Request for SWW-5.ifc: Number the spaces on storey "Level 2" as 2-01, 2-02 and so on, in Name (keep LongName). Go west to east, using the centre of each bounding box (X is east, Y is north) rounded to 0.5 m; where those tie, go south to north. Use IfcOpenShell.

First a look at what the model holds.

```python
import ifcopenshell
import ifcopenshell.util.element
import ifcopenshell.util.placement

model = ifcopenshell.open("SWW-5.ifc")
print(model.schema)
storey = next(s for s in model.by_type("IfcBuildingStorey") if s.Name == "Level 2")
spaces = [e for e in ifcopenshell.util.element.get_decomposition(storey) if e.is_a("IfcSpace")]
for e in sorted(spaces, key=lambda e: e.id()):
    origin = ifcopenshell.util.placement.get_local_placement(e.ObjectPlacement)[:3, 3]
    print(e.id(), e.Name, e.LongName, origin.round(2) + 0.0, sep=" | ")
```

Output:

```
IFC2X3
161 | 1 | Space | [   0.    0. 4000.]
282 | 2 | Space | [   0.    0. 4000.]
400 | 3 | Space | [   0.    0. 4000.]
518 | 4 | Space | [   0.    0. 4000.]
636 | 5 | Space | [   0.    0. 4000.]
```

```python
import ifcopenshell
import ifcopenshell.geom
import ifcopenshell.util.element
import ifcopenshell.util.shape

model = ifcopenshell.open("SWW-5.ifc")
settings = ifcopenshell.geom.settings()
settings.set("use-world-coords", True)


def centre(element):
    shape = ifcopenshell.geom.create_shape(settings, element)
    return ifcopenshell.util.shape.get_bbox_centroid(shape.geometry)


storey = next(s for s in model.by_type("IfcBuildingStorey") if s.Name == "Level 2")
spaces = [e for e in ifcopenshell.util.element.get_decomposition(storey) if e.is_a("IfcSpace")]

# Insertion points can sit at a corner or the storey origin, so sort by the geometry (in metres).
centres = {e: centre(e) for e in spaces}
spaces.sort(key=lambda e: (round(centres[e][0] / 0.5), centres[e][1]))

for i, e in enumerate(spaces, start=1):
    number = f"2-{i:02d}"
    e.Name = number
    print(e.id(), number)

model.write("SWW-5_updated.ifc")
```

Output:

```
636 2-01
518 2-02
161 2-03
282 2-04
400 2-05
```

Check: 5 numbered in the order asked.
